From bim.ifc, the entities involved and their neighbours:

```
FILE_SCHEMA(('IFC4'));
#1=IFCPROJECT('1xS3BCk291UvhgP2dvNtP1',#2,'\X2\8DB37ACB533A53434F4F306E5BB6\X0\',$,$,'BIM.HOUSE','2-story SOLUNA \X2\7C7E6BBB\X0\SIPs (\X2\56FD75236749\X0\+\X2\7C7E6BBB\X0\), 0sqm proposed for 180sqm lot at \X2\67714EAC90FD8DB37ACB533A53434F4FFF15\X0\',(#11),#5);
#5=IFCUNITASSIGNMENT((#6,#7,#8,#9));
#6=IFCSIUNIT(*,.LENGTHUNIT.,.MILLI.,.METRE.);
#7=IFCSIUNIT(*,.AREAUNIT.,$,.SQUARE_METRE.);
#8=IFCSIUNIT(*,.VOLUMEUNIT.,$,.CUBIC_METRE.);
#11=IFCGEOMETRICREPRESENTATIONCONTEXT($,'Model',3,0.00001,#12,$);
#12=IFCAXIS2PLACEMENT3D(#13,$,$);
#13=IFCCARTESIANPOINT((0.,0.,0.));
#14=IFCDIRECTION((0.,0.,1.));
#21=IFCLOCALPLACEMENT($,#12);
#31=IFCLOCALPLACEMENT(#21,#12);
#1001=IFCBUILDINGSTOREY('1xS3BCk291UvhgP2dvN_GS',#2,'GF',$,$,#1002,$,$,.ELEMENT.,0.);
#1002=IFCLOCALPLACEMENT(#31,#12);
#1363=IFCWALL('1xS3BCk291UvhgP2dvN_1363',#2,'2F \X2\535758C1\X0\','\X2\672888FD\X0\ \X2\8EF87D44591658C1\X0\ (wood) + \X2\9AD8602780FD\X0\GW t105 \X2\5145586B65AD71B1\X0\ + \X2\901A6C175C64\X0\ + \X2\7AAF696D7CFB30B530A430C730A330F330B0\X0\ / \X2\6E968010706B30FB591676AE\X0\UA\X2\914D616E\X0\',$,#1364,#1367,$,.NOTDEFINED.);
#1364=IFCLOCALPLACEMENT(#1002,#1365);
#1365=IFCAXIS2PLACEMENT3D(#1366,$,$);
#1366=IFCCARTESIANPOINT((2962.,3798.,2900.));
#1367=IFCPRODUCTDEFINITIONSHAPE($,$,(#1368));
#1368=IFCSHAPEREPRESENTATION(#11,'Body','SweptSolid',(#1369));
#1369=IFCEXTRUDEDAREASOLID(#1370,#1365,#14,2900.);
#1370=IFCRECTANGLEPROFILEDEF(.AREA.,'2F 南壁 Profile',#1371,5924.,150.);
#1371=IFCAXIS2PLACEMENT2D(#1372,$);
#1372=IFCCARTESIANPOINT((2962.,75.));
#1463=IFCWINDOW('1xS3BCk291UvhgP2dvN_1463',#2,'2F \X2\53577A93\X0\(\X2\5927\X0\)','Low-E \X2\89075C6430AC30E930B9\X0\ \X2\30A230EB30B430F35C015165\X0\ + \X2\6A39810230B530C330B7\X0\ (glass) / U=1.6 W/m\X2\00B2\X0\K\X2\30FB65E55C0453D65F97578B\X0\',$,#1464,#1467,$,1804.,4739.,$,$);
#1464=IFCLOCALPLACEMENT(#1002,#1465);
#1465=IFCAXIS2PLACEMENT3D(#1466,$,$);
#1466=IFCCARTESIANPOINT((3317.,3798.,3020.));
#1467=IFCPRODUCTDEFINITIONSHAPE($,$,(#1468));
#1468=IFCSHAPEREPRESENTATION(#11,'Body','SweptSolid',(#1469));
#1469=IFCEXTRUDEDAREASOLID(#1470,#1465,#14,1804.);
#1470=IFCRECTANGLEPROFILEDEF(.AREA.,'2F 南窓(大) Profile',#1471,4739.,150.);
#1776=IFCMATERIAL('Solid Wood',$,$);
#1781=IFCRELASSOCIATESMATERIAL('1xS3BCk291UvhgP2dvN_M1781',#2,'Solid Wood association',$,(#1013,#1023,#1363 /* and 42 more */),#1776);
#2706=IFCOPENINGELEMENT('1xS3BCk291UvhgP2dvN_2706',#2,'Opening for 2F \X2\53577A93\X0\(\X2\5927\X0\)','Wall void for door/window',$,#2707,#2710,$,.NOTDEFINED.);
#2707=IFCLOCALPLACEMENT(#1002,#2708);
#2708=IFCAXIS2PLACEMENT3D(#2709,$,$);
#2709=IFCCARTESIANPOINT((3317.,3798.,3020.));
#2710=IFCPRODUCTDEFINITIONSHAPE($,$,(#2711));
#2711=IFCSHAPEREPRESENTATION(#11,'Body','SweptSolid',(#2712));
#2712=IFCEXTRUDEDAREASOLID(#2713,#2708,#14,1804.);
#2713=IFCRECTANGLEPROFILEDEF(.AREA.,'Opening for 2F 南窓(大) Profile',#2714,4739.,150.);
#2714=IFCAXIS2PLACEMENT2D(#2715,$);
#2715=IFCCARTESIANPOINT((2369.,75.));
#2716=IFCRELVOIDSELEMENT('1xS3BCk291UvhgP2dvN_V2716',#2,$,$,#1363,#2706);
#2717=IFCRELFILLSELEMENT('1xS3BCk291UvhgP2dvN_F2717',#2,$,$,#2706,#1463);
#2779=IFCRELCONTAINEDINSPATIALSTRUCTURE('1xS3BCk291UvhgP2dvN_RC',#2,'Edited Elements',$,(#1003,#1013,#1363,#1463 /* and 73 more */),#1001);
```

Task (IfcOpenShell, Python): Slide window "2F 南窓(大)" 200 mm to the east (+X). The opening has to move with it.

```python
import ifcopenshell
import ifcopenshell.api.geometry
import ifcopenshell.util.placement
import ifcopenshell.util.unit

model = ifcopenshell.open("bim.ifc")
unit_scale = ifcopenshell.util.unit.calculate_unit_scale(model)

window = model.by_guid("1xS3BCk291UvhgP2dvN_1463")
opening = window.FillsVoids[0].RelatingOpeningElement
wall = opening.VoidsElements[0].RelatingBuildingElement

wall_matrix = ifcopenshell.util.placement.get_local_placement(wall.ObjectPlacement)
shift = wall_matrix[:3, 0] * 0.2 / unit_scale
before = ifcopenshell.util.placement.get_local_placement(window.ObjectPlacement)[:3, 3].copy()

# The window is not placed relative to its opening, so move both.
for product in (opening, window):
    matrix = ifcopenshell.util.placement.get_local_placement(product.ObjectPlacement)
    matrix[:3, 3] += shift
    ifcopenshell.api.geometry.edit_object_placement(model, product=product, matrix=matrix, is_si=False)

after = ifcopenshell.util.placement.get_local_placement(window.ObjectPlacement)[:3, 3]
print("window moved by", (after - before).round(3) + 0.0)

model.write("bim_v2.ifc")
```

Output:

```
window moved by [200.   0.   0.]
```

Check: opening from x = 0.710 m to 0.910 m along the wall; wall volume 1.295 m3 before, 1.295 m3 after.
